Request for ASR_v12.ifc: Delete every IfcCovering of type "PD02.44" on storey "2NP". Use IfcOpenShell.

First a look at what the model holds.

```python
import ifcopenshell
import ifcopenshell.util.element

model = ifcopenshell.open("ASR_v12.ifc")
print(model.schema)
storey = next(s for s in model.by_type("IfcBuildingStorey") if s.Name == "2NP")
coverings = [e for e in ifcopenshell.util.element.get_decomposition(storey) if e.is_a("IfcCovering")]
seen = {}
for e in coverings:
    element_type = ifcopenshell.util.element.get_type(e)
    name = element_type.Name if element_type not in (None, e) else None
    seen[name] = seen.get(name, 0) + 1
for name, count in sorted(seen.items(), key=str):
    print(count, "x", name)
```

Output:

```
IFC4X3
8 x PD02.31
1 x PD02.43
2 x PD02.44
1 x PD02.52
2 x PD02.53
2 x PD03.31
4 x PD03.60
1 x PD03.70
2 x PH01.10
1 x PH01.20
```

```python
import ifcopenshell
import ifcopenshell.api.root
import ifcopenshell.util.element

model = ifcopenshell.open("ASR_v12.ifc")

storey = next(s for s in model.by_type("IfcBuildingStorey") if s.Name == "2NP")
coverings = [e for e in ifcopenshell.util.element.get_decomposition(storey) if e.is_a("IfcCovering")]
targets = [e for e in coverings if (t := ifcopenshell.util.element.get_type(e)) not in (None, e) and t.Name == "PD02.44"]

for e in targets:
    ifcopenshell.api.root.remove_product(model, product=e)
print(len(targets), "removed")

model.write("ASR_v12_rev.ifc")
```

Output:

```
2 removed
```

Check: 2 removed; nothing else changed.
